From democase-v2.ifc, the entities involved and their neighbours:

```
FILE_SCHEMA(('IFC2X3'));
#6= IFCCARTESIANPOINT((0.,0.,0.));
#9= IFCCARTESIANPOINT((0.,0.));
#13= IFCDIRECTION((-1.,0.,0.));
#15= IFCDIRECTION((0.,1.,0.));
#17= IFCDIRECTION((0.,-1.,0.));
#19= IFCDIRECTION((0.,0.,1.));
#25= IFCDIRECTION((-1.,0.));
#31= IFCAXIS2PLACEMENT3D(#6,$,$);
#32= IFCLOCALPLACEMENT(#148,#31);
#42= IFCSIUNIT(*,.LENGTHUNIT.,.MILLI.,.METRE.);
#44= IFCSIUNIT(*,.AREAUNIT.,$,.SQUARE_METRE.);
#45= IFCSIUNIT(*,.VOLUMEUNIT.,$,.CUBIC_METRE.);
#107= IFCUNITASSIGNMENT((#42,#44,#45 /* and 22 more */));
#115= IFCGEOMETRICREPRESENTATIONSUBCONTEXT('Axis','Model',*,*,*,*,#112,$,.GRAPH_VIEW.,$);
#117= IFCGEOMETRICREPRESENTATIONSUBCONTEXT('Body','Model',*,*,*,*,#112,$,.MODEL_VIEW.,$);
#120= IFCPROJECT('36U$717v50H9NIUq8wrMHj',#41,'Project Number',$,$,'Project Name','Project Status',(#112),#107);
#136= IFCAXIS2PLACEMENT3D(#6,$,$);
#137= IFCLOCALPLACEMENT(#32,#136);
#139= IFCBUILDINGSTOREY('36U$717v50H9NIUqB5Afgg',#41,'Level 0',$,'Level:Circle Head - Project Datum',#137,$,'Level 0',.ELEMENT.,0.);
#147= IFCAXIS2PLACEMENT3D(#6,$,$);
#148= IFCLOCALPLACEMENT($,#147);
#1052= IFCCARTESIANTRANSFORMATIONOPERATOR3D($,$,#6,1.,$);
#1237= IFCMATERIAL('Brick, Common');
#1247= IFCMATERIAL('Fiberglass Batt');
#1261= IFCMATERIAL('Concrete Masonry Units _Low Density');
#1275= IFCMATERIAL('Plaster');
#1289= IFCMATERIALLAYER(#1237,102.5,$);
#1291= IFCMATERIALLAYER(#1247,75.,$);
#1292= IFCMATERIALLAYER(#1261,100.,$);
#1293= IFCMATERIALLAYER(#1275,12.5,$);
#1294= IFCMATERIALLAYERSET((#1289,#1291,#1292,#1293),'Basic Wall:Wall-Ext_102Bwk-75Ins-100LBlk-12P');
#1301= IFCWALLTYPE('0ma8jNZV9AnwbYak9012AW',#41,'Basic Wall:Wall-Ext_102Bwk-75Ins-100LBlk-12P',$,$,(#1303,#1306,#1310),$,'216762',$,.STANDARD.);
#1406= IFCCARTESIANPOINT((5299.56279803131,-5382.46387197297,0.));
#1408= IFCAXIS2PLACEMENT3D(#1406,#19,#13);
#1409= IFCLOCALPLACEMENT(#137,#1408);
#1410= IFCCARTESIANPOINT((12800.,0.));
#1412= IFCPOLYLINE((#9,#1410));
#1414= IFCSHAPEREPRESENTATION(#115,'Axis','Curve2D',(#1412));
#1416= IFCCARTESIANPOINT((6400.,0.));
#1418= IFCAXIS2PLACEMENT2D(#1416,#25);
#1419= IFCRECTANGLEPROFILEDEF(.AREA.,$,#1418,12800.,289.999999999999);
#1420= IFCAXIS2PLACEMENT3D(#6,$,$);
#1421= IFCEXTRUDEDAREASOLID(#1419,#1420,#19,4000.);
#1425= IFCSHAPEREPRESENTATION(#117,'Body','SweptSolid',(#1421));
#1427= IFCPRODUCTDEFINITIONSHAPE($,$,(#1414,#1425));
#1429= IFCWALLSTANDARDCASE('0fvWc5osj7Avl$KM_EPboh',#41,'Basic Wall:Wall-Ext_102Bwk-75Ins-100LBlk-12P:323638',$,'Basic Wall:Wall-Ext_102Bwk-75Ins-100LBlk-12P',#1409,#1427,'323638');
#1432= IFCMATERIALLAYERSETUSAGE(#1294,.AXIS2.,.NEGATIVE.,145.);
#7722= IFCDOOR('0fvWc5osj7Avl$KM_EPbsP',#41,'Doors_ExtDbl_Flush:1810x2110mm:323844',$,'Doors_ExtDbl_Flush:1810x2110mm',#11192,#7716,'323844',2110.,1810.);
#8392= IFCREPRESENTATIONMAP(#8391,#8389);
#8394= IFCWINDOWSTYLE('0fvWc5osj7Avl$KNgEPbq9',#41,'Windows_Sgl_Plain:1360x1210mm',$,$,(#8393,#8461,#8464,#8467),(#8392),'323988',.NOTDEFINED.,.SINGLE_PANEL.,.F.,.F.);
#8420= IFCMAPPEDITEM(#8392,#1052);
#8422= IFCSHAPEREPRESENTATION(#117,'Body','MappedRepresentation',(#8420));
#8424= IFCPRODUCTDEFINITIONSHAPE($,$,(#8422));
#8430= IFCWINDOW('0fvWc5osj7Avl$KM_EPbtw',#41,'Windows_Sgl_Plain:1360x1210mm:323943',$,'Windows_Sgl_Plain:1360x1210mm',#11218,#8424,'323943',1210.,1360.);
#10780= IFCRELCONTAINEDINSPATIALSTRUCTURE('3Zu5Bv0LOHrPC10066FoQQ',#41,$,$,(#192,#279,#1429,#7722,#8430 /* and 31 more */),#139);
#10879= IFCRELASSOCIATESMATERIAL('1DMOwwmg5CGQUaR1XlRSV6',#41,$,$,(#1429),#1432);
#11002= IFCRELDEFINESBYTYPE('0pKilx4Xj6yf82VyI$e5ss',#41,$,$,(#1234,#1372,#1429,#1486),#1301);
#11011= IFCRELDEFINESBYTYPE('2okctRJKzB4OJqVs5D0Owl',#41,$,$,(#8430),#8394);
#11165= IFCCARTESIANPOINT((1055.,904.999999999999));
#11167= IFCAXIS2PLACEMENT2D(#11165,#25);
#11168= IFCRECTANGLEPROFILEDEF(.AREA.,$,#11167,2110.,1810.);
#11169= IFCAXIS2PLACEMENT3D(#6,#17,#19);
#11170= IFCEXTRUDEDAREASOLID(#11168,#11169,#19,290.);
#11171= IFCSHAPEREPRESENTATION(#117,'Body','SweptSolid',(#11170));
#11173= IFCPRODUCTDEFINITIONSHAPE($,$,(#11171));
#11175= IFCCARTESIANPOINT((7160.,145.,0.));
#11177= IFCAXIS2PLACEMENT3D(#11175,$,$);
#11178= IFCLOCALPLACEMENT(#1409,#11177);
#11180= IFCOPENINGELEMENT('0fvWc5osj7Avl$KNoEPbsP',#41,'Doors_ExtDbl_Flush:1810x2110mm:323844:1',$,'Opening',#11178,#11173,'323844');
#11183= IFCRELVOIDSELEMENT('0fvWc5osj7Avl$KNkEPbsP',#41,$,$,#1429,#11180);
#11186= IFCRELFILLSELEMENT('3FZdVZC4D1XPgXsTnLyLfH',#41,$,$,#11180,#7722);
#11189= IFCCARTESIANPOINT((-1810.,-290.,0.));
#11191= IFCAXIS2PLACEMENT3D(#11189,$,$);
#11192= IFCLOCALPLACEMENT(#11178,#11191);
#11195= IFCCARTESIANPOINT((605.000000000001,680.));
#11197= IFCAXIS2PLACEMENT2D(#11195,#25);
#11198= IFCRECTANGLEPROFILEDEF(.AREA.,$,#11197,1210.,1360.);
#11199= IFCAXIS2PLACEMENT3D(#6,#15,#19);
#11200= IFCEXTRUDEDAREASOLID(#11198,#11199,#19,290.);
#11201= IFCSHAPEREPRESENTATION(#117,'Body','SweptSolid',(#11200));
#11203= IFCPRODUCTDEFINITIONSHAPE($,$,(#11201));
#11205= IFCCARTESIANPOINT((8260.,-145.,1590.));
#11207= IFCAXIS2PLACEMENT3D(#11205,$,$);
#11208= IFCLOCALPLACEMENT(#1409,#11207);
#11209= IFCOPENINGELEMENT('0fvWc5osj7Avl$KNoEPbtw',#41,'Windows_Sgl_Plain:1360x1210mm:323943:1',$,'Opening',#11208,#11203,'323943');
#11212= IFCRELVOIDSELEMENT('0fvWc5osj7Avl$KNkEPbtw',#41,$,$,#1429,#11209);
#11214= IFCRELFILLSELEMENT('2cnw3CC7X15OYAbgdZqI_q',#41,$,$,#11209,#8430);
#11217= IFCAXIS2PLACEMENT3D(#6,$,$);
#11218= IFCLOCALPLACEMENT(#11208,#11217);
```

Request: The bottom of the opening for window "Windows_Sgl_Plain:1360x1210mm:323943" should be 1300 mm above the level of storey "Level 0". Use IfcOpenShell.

```python
import numpy as np
import ifcopenshell
import ifcopenshell.api.geometry
import ifcopenshell.geom
import ifcopenshell.util.element
import ifcopenshell.util.placement
import ifcopenshell.util.shape
import ifcopenshell.util.unit

model = ifcopenshell.open("democase-v2.ifc")
unit_scale = ifcopenshell.util.unit.calculate_unit_scale(model)

window = model.by_guid("0fvWc5osj7Avl$KM_EPbtw")
opening = window.FillsVoids[0].RelatingOpeningElement
storey = ifcopenshell.util.element.get_container(window, ifc_class="IfcBuildingStorey")
level = ifcopenshell.util.placement.get_local_placement(storey.ObjectPlacement)[2, 3]

# The opening's origin need not be at the sill, so measure its lowest point.
shape = ifcopenshell.geom.create_shape(ifcopenshell.geom.settings(), opening)
bottom = ifcopenshell.util.shape.get_shape_bottom_elevation(shape, shape.geometry) / unit_scale
dz = level + 1300.0 - bottom

shift = np.array([0.0, 0.0, dz])
# The window is placed relative to its opening, so it follows when the opening moves.
matrix = ifcopenshell.util.placement.get_local_placement(opening.ObjectPlacement)
matrix[:3, 3] += shift
ifcopenshell.api.geometry.edit_object_placement(
    model, product=opening, matrix=matrix, is_si=False, should_transform_children=True
)

print(f"moved by {dz * unit_scale:+.3f} m")

model.write("democase-v2-out.ifc")
```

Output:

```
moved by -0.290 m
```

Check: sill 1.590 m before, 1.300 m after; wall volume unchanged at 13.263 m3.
